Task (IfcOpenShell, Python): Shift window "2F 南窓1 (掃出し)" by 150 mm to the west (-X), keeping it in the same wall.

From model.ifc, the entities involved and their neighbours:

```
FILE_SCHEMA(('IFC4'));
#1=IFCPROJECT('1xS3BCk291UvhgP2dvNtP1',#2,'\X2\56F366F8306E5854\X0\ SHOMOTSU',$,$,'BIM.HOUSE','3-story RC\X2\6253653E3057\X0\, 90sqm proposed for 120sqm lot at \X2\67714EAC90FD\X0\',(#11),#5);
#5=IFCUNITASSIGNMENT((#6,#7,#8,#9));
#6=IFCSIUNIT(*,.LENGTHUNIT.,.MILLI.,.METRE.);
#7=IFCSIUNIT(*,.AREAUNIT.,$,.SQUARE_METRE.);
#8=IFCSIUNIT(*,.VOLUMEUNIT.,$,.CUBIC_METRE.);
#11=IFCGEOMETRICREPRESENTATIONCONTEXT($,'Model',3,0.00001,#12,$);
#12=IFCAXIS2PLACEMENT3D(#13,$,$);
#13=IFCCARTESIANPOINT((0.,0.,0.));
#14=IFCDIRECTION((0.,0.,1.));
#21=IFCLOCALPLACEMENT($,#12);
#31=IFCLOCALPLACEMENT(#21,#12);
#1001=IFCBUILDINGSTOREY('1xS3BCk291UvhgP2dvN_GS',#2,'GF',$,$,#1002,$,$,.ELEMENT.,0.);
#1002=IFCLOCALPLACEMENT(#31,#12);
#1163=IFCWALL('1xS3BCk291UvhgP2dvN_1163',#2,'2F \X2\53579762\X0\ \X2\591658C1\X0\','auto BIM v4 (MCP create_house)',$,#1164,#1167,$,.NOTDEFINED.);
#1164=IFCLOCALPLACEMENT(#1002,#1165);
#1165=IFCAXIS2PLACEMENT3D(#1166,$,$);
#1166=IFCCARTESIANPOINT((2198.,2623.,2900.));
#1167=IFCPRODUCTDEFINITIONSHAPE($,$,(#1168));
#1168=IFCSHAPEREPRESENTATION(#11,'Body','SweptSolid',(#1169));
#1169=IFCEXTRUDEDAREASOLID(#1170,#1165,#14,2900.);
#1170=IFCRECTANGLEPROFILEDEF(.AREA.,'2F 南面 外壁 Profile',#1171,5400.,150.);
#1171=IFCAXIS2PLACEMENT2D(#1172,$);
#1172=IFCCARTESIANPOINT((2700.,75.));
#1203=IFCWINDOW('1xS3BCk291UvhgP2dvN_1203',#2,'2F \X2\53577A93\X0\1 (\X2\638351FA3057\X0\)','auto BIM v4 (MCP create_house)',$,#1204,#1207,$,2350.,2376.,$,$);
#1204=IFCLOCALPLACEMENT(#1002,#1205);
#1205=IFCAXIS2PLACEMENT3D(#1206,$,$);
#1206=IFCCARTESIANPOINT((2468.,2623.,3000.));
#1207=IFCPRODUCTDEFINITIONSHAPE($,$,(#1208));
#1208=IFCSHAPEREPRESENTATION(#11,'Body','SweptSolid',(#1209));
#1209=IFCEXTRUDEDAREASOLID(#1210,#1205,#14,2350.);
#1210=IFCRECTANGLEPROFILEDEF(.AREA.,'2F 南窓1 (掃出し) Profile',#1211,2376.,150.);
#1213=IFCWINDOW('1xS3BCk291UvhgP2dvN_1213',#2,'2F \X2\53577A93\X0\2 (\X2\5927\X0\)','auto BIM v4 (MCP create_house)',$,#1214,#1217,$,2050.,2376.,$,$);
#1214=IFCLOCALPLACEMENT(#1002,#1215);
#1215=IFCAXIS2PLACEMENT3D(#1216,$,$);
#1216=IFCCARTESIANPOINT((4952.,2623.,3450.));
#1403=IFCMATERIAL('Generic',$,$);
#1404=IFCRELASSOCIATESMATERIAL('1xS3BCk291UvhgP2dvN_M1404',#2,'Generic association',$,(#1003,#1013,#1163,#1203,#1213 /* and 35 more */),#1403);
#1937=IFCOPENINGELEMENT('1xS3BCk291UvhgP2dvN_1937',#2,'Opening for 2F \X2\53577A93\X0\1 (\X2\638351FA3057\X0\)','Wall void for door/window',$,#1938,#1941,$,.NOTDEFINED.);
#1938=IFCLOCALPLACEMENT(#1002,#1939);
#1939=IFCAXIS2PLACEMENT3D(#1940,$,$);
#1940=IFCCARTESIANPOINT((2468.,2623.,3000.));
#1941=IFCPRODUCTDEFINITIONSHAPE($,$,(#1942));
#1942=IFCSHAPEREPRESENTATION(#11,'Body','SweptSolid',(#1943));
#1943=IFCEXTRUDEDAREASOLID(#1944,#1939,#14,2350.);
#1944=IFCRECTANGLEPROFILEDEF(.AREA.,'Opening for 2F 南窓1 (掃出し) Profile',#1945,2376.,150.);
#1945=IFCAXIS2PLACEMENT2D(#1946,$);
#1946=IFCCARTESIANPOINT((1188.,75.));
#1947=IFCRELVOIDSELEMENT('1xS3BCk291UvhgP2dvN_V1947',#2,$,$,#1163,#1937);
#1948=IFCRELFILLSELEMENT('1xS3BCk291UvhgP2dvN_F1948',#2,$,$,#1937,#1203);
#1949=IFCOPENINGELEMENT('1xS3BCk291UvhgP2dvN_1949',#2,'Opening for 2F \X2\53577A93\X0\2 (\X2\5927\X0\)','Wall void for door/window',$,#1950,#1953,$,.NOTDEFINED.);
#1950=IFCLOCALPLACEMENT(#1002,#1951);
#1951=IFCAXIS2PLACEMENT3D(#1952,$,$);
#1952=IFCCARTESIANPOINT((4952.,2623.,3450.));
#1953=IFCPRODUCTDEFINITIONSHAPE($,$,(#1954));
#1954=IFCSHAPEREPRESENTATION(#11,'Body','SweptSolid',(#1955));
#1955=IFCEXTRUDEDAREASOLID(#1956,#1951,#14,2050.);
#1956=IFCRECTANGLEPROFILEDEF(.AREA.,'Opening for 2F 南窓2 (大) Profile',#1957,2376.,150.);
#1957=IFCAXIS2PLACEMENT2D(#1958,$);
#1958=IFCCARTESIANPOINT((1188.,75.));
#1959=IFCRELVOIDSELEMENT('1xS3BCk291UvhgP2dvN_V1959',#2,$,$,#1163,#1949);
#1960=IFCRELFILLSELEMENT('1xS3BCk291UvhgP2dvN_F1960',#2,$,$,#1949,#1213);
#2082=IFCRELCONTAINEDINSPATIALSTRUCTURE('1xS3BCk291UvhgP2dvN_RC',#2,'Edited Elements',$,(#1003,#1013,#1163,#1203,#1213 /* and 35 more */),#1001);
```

```python
import ifcopenshell
import ifcopenshell.api.geometry
import ifcopenshell.util.placement
import ifcopenshell.util.unit

model = ifcopenshell.open("model.ifc")
unit_scale = ifcopenshell.util.unit.calculate_unit_scale(model)

window = model.by_guid("1xS3BCk291UvhgP2dvN_1203")
opening = window.FillsVoids[0].RelatingOpeningElement
wall = opening.VoidsElements[0].RelatingBuildingElement

wall_matrix = ifcopenshell.util.placement.get_local_placement(wall.ObjectPlacement)
shift = wall_matrix[:3, 0] * -0.15 / unit_scale
before = ifcopenshell.util.placement.get_local_placement(window.ObjectPlacement)[:3, 3].copy()

# The window is not placed relative to its opening, so move both.
for product in (opening, window):
    matrix = ifcopenshell.util.placement.get_local_placement(product.ObjectPlacement)
    matrix[:3, 3] += shift
    ifcopenshell.api.geometry.edit_object_placement(model, product=product, matrix=matrix, is_si=False)

after = ifcopenshell.util.placement.get_local_placement(window.ObjectPlacement)[:3, 3]
print("window moved by", (after - before).round(3) + 0.0)

model.write("model_rev.ifc")
```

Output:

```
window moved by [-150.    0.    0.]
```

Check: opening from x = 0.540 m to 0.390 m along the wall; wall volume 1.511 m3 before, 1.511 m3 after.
